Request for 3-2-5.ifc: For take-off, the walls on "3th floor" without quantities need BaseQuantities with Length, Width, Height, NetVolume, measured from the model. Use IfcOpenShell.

First a look at what the model holds.

```python
import ifcopenshell
import ifcopenshell.util.element
import ifcopenshell.util.unit

model = ifcopenshell.open("3-2-5.ifc")
print(model.schema)
for unit_type in ("LENGTHUNIT", "AREAUNIT", "VOLUMEUNIT"):
    print(unit_type, ifcopenshell.util.unit.calculate_unit_scale(model, unit_type))
storey = next(s for s in model.by_type("IfcBuildingStorey") if s.Name == "3th floor")
walls = [e for e in ifcopenshell.util.element.get_decomposition(storey) if e.is_a("IfcWall")]
for e in sorted(walls, key=lambda e: e.id()):
    print(e.id(), e.is_a(), e.Name, list(ifcopenshell.util.element.get_psets(e, qtos_only=True)), sep=" | ")
```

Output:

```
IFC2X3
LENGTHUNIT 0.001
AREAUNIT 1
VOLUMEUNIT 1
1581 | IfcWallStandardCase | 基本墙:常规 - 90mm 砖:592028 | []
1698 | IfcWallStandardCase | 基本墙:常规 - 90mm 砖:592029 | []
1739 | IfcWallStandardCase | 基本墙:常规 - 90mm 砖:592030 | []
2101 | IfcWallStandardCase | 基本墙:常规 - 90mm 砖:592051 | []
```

```python
import ifcopenshell
import ifcopenshell.api.pset
import ifcopenshell.geom
import ifcopenshell.util.element
import ifcopenshell.util.shape
import ifcopenshell.util.unit

model = ifcopenshell.open("3-2-5.ifc")
unit_scale = ifcopenshell.util.unit.calculate_unit_scale(model)
volume_scale = ifcopenshell.util.unit.calculate_unit_scale(model, "VOLUMEUNIT")
settings = ifcopenshell.geom.settings()

storey = next(s for s in model.by_type("IfcBuildingStorey") if s.Name == "3th floor")
walls = [e for e in ifcopenshell.util.element.get_decomposition(storey) if e.is_a("IfcWall")]

for e in sorted(walls, key=lambda e: e.id()):
    if ifcopenshell.util.element.get_psets(e, qtos_only=True, should_inherit=False):
        continue
    # Geometry comes back in metres, in the element's own axes.
    shape = ifcopenshell.geom.create_shape(settings, e)
    values = {
        "Length": ifcopenshell.util.shape.get_x(shape.geometry) / unit_scale,
        "Width": ifcopenshell.util.shape.get_y(shape.geometry) / unit_scale,
        "Height": ifcopenshell.util.shape.get_z(shape.geometry) / unit_scale,
        "NetVolume": ifcopenshell.util.shape.get_volume(shape.geometry) / volume_scale,
    }
    qto = ifcopenshell.api.pset.add_qto(model, product=e, name="BaseQuantities")
    ifcopenshell.api.pset.edit_qto(model, qto=qto, properties=values)
    print(e.id(), {k: round(v, 3) for k, v in values.items()})

model.write("3-2-5_updated.ifc")
```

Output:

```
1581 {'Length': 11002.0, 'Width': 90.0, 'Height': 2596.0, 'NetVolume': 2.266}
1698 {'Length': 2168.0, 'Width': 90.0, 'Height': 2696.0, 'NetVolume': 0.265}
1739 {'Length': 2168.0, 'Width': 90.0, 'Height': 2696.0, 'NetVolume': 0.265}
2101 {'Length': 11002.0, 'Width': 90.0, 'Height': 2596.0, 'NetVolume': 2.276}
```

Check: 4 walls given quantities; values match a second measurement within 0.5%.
